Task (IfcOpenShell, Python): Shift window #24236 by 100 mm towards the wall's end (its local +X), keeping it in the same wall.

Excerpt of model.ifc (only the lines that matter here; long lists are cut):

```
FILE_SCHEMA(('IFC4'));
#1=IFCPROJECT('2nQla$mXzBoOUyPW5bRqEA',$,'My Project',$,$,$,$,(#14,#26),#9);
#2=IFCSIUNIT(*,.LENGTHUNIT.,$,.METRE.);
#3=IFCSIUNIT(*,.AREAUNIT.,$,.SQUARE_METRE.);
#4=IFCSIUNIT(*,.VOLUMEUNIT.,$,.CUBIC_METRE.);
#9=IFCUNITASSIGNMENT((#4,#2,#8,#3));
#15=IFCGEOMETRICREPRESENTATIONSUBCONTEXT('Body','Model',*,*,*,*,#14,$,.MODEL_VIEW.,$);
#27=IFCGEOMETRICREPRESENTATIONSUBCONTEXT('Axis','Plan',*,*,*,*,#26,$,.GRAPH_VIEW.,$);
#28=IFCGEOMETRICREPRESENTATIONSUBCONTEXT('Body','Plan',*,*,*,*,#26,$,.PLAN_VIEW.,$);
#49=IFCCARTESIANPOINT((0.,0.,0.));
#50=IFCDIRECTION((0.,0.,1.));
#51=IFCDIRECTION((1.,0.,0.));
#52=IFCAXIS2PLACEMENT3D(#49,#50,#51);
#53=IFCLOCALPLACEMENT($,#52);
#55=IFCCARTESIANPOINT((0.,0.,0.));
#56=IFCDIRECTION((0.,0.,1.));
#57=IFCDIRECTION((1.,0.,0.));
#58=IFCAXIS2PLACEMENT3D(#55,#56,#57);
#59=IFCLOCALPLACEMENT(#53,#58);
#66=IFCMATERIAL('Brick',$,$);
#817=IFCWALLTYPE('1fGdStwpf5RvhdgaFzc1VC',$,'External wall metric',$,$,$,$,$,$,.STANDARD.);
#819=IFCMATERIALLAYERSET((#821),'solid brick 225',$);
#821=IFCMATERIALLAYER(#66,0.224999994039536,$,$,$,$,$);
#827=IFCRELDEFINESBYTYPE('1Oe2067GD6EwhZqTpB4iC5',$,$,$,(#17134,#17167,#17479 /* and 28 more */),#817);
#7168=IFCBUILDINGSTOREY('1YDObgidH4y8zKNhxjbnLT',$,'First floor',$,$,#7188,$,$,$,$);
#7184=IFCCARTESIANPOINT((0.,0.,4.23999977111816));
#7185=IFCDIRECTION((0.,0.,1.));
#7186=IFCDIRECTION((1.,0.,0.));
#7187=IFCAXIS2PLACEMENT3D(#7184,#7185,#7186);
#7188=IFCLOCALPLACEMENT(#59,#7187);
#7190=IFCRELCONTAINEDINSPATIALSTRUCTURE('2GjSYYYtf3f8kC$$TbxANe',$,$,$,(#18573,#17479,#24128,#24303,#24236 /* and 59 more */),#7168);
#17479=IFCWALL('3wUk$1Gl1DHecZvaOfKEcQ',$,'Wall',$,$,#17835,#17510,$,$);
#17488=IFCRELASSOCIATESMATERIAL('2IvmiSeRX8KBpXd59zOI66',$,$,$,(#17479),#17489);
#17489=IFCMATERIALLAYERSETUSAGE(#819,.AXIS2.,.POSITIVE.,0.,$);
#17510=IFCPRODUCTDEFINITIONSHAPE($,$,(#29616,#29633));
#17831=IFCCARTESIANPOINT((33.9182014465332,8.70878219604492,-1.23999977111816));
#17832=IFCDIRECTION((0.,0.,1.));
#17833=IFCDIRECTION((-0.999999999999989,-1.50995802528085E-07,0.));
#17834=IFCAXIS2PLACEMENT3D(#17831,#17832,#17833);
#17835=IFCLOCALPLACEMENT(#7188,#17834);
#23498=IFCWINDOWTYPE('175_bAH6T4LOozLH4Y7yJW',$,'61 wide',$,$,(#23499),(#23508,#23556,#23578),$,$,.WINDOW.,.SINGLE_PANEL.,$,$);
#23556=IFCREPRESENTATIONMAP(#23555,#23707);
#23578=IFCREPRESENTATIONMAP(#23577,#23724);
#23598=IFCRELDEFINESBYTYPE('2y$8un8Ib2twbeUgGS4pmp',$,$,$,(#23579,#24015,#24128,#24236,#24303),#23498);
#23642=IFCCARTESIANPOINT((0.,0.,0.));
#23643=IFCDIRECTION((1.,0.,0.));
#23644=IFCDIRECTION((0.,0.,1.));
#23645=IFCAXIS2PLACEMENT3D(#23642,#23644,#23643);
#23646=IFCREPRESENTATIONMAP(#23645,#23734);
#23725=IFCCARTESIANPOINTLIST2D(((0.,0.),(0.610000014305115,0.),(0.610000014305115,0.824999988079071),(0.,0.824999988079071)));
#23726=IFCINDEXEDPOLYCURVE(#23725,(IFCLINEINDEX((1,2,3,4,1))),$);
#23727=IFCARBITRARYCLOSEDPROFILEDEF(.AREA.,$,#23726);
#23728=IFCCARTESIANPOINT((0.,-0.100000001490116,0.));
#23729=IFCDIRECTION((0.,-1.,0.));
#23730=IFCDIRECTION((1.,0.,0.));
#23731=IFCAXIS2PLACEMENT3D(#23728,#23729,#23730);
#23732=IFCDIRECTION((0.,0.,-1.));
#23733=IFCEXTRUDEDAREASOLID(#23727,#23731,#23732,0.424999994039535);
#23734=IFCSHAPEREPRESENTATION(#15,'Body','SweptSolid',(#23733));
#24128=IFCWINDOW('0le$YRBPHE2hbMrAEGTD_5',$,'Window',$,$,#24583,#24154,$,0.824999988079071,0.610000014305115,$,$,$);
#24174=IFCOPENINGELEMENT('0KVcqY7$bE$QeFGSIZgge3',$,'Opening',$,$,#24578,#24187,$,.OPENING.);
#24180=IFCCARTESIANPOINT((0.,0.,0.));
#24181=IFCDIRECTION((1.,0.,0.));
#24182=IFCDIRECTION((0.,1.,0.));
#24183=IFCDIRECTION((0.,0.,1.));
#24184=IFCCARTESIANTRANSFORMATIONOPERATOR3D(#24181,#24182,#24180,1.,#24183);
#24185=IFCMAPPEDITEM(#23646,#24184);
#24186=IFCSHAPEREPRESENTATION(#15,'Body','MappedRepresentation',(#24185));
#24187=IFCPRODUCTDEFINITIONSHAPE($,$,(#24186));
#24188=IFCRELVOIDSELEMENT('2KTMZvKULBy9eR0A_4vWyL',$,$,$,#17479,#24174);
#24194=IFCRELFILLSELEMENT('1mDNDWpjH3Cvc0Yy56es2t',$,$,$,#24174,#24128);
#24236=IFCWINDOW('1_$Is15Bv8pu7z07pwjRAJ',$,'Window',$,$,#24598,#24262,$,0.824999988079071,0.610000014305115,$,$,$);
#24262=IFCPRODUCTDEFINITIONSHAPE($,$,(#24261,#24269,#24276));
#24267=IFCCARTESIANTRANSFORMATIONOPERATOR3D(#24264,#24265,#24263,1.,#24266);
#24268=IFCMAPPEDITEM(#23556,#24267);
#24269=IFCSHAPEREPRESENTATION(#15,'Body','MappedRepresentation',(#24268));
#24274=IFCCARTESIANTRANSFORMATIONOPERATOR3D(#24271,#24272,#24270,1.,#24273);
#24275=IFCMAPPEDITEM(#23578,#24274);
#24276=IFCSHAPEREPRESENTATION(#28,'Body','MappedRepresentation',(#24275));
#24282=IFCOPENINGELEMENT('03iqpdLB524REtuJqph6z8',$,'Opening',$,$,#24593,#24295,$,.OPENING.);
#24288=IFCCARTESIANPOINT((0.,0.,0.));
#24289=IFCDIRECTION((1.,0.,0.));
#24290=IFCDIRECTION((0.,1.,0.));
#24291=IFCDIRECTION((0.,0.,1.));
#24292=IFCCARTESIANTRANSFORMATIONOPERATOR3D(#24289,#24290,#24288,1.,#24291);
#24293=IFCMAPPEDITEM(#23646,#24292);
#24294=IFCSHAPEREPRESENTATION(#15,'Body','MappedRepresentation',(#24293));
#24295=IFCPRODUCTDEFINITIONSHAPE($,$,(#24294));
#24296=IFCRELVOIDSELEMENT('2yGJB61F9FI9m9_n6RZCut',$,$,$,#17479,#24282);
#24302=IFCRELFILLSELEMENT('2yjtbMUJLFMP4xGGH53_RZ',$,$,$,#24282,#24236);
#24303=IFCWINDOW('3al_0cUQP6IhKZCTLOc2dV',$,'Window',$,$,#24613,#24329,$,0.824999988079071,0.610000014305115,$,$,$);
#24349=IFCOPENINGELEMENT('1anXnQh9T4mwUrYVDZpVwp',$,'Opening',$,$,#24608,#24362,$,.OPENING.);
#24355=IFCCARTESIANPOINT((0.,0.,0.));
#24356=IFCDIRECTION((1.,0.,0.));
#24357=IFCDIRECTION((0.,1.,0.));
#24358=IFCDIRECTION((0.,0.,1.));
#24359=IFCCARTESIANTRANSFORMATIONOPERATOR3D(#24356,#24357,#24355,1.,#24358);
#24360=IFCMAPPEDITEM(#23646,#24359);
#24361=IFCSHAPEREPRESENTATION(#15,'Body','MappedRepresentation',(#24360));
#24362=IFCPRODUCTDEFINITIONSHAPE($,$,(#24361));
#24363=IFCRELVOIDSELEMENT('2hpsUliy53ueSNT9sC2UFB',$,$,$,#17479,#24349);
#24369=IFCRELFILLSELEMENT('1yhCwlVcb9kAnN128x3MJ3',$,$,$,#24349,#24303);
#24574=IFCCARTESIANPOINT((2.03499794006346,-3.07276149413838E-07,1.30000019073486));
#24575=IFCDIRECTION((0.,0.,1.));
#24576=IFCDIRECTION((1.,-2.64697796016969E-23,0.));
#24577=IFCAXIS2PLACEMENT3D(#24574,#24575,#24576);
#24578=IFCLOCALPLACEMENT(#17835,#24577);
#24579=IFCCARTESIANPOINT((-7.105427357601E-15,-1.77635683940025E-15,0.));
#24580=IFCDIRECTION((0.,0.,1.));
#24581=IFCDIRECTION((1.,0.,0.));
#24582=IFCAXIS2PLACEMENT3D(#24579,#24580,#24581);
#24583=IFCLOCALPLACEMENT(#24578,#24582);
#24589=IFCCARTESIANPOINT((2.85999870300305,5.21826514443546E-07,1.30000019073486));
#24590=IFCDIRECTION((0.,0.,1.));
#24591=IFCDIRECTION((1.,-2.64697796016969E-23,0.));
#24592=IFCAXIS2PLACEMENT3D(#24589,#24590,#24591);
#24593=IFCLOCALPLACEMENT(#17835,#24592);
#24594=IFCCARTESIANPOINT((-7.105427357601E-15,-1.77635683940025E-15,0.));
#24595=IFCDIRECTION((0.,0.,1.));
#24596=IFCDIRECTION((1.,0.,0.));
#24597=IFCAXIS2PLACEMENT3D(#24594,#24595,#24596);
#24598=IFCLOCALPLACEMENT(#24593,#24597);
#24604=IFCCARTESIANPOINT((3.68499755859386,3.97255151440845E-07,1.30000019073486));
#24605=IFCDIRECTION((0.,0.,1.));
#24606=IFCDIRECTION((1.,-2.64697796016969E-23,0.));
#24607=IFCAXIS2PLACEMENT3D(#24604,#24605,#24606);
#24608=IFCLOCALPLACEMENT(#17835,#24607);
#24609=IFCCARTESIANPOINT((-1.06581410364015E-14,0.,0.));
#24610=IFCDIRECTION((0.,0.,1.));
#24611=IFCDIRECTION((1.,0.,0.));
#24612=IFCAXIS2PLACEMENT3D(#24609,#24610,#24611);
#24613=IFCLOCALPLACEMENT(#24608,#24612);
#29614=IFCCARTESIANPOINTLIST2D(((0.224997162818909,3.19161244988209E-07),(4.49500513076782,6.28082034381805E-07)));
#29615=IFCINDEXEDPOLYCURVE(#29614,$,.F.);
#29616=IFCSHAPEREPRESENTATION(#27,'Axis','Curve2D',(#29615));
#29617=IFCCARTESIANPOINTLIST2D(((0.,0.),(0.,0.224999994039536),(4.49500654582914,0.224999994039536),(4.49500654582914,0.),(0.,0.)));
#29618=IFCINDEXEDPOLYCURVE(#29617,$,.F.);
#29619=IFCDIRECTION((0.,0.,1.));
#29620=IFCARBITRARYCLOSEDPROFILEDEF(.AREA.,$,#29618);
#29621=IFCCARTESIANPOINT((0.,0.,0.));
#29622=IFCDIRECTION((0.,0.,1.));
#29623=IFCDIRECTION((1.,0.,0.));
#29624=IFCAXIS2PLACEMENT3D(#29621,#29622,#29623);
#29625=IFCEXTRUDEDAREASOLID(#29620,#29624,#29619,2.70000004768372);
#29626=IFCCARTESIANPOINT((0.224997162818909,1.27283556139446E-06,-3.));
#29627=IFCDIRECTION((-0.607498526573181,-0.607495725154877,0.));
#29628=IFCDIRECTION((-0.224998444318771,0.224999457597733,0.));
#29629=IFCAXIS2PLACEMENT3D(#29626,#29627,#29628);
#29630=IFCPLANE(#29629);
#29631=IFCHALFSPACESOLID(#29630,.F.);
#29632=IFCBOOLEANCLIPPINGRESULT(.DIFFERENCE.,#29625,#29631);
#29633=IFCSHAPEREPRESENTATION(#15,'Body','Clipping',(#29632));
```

```python
import ifcopenshell
import ifcopenshell.api.geometry
import ifcopenshell.util.placement

model = ifcopenshell.open("model.ifc")

window = model.by_id(24236)
opening = window.FillsVoids[0].RelatingOpeningElement
wall = opening.VoidsElements[0].RelatingBuildingElement

wall_matrix = ifcopenshell.util.placement.get_local_placement(wall.ObjectPlacement)
shift = wall_matrix[:3, 0] * 0.1
before = ifcopenshell.util.placement.get_local_placement(window.ObjectPlacement)[:3, 3].copy()

# The window is placed relative to its opening, so it follows when the opening moves.
matrix = ifcopenshell.util.placement.get_local_placement(opening.ObjectPlacement)
matrix[:3, 3] += shift
ifcopenshell.api.geometry.edit_object_placement(
    model, product=opening, matrix=matrix, is_si=False, should_transform_children=True
)

after = ifcopenshell.util.placement.get_local_placement(window.ObjectPlacement)[:3, 3]
print("window moved by", (after - before).round(3) + 0.0)

model.write("model_updated.ifc")
```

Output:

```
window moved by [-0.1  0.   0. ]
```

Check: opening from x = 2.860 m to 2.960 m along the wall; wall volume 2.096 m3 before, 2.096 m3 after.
